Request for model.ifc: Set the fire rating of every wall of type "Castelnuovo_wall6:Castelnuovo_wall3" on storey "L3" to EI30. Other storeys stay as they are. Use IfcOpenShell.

First a look at what the model holds.

```python
import ifcopenshell
import ifcopenshell.util.element

model = ifcopenshell.open("model.ifc")
print(model.schema)
storey = next(s for s in model.by_type("IfcBuildingStorey") if s.Name == "L3")
walls = [e for e in ifcopenshell.util.element.get_decomposition(storey) if e.is_a("IfcWall")]
seen = {}
for e in walls:
    element_type = ifcopenshell.util.element.get_type(e)
    key = (element_type.Name if element_type != e and element_type else None, ifcopenshell.util.element.get_pset(e, "Pset_WallCommon", "FireRating"))
    seen[key] = seen.get(key, 0) + 1
for (name, value), count in sorted(seen.items(), key=str):
    print(count, "x", name, "|", value)
```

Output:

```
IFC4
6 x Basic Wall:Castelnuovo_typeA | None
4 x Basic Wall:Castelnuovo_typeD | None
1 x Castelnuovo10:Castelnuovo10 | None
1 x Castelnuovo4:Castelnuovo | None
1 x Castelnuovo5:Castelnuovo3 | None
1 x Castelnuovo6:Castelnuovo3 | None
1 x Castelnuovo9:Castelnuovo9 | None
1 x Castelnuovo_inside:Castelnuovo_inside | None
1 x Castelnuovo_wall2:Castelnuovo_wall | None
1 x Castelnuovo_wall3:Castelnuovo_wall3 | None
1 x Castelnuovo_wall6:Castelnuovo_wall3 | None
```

```python
import ifcopenshell
import ifcopenshell.api.pset
import ifcopenshell.util.element

model = ifcopenshell.open("model.ifc")

storey = next(s for s in model.by_type("IfcBuildingStorey") if s.Name == "L3")
walls = [e for e in ifcopenshell.util.element.get_decomposition(storey) if e.is_a("IfcWall")]

count = 0
for e in walls:
    element_type = ifcopenshell.util.element.get_type(e)
    if element_type in (None, e) or element_type.Name != "Castelnuovo_wall6:Castelnuovo_wall3":
        continue
    # add_pset returns the element's existing set when there is one.
    pset = ifcopenshell.api.pset.add_pset(model, product=e, name="Pset_WallCommon")
    ifcopenshell.api.pset.edit_pset(model, pset=pset, properties={"FireRating": "EI30"})
    count += 1

print(count, "walls updated")

model.write("model-out.ifc")
```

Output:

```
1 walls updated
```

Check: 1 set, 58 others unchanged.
